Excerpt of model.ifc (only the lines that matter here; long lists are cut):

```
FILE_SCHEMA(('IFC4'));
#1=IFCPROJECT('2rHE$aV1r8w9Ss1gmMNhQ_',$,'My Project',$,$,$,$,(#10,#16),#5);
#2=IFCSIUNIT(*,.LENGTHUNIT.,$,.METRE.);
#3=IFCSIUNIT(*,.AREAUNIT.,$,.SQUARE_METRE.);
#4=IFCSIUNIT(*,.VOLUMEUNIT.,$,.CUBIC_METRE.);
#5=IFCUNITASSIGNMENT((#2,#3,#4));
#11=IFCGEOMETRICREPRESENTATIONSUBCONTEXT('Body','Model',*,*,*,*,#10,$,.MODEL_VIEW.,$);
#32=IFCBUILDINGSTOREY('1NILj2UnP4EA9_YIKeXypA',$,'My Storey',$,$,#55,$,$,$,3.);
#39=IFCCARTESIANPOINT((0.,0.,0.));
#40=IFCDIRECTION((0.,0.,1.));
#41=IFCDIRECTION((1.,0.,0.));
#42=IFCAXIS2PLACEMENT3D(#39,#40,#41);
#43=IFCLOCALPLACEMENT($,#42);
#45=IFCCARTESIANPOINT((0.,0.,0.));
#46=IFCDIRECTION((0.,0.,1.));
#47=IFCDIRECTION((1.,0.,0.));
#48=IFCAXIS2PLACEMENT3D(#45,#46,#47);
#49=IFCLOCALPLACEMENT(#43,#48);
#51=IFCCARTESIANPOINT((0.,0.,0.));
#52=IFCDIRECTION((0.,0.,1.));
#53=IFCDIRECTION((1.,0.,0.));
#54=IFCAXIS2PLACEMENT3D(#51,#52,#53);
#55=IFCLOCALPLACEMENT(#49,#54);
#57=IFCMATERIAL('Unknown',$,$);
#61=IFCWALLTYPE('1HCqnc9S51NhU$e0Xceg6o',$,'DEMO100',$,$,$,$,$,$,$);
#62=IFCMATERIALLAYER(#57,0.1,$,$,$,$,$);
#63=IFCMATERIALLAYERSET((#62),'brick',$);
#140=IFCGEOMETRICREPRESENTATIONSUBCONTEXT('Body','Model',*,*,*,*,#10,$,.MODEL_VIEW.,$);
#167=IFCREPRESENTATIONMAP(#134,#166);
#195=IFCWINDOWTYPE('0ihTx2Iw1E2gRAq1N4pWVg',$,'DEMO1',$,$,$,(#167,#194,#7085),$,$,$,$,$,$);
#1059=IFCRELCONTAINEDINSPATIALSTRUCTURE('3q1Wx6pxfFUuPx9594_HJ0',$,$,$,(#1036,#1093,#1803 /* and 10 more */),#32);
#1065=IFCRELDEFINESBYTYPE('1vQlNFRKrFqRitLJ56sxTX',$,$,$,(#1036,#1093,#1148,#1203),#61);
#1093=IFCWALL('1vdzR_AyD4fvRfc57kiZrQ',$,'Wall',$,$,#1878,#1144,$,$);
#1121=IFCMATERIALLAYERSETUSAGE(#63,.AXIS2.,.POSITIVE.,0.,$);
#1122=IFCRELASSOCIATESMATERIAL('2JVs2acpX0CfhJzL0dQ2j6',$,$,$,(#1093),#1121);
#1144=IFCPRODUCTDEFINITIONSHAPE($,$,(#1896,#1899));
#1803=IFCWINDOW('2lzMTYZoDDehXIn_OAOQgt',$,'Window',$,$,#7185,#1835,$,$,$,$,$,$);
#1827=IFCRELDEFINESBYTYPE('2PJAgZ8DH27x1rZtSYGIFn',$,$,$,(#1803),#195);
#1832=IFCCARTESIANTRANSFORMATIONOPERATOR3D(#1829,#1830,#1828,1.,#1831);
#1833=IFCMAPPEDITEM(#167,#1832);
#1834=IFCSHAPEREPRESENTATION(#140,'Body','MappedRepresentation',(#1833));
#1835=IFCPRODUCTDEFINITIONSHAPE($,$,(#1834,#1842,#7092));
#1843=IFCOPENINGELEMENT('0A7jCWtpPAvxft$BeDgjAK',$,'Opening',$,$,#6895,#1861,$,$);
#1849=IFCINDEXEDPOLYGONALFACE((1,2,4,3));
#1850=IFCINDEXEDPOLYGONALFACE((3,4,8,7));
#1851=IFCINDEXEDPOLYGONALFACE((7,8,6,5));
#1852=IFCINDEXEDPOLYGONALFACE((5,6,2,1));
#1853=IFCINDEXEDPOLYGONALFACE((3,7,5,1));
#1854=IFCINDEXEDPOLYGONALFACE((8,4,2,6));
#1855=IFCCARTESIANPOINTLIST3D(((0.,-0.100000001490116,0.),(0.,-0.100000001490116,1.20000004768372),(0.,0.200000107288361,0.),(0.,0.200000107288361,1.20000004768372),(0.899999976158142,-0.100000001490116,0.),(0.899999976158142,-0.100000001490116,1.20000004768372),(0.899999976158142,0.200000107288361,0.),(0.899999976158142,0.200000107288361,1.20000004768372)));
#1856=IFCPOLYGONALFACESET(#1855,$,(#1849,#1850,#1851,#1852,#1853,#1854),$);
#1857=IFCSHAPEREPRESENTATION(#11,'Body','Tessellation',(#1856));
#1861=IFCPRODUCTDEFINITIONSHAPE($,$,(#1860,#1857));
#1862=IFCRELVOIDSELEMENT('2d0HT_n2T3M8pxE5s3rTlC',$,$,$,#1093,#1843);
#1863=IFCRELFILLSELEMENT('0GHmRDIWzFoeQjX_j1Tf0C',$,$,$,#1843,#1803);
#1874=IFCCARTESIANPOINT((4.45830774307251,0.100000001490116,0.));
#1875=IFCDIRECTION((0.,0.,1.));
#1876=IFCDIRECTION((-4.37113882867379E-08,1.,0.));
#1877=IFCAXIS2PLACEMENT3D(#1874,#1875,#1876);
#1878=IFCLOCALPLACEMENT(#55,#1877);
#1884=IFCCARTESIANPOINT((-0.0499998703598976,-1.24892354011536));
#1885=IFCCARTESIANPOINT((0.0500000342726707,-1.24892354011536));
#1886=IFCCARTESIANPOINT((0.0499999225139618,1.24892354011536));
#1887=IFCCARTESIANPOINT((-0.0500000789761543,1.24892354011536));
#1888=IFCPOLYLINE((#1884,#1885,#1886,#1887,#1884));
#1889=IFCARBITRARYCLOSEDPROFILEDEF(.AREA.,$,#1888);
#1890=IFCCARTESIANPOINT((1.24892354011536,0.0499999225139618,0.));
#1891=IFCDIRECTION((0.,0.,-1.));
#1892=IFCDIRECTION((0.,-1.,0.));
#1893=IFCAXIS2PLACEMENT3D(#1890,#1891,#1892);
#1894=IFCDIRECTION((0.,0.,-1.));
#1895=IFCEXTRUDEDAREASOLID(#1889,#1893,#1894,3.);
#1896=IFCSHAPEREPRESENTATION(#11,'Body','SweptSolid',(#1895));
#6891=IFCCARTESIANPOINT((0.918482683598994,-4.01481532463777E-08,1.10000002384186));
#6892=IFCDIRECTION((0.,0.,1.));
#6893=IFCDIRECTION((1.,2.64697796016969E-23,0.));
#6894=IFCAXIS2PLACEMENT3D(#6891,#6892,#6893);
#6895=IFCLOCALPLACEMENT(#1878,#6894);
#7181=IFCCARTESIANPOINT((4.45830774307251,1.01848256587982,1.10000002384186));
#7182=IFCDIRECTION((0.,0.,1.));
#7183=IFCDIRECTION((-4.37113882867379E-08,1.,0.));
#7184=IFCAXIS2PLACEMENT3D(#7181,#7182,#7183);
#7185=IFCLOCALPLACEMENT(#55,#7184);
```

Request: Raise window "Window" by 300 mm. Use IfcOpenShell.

```python
import numpy as np
import ifcopenshell
import ifcopenshell.api.geometry
import ifcopenshell.util.placement
import ifcopenshell.util.unit

model = ifcopenshell.open("model.ifc")
unit_scale = ifcopenshell.util.unit.calculate_unit_scale(model)

window = model.by_guid("2lzMTYZoDDehXIn_OAOQgt")
opening = window.FillsVoids[0].RelatingOpeningElement
dz = 0.3

shift = np.array([0.0, 0.0, dz])
# The window is not placed relative to its opening, so move both.
for product in (opening, window):
    matrix = ifcopenshell.util.placement.get_local_placement(product.ObjectPlacement)
    matrix[:3, 3] += shift
    ifcopenshell.api.geometry.edit_object_placement(model, product=product, matrix=matrix, is_si=False)

print(f"moved by {dz * unit_scale:+.3f} m")

model.write("model_updated.ifc")
```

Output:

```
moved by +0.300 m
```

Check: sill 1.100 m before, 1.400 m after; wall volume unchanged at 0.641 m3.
